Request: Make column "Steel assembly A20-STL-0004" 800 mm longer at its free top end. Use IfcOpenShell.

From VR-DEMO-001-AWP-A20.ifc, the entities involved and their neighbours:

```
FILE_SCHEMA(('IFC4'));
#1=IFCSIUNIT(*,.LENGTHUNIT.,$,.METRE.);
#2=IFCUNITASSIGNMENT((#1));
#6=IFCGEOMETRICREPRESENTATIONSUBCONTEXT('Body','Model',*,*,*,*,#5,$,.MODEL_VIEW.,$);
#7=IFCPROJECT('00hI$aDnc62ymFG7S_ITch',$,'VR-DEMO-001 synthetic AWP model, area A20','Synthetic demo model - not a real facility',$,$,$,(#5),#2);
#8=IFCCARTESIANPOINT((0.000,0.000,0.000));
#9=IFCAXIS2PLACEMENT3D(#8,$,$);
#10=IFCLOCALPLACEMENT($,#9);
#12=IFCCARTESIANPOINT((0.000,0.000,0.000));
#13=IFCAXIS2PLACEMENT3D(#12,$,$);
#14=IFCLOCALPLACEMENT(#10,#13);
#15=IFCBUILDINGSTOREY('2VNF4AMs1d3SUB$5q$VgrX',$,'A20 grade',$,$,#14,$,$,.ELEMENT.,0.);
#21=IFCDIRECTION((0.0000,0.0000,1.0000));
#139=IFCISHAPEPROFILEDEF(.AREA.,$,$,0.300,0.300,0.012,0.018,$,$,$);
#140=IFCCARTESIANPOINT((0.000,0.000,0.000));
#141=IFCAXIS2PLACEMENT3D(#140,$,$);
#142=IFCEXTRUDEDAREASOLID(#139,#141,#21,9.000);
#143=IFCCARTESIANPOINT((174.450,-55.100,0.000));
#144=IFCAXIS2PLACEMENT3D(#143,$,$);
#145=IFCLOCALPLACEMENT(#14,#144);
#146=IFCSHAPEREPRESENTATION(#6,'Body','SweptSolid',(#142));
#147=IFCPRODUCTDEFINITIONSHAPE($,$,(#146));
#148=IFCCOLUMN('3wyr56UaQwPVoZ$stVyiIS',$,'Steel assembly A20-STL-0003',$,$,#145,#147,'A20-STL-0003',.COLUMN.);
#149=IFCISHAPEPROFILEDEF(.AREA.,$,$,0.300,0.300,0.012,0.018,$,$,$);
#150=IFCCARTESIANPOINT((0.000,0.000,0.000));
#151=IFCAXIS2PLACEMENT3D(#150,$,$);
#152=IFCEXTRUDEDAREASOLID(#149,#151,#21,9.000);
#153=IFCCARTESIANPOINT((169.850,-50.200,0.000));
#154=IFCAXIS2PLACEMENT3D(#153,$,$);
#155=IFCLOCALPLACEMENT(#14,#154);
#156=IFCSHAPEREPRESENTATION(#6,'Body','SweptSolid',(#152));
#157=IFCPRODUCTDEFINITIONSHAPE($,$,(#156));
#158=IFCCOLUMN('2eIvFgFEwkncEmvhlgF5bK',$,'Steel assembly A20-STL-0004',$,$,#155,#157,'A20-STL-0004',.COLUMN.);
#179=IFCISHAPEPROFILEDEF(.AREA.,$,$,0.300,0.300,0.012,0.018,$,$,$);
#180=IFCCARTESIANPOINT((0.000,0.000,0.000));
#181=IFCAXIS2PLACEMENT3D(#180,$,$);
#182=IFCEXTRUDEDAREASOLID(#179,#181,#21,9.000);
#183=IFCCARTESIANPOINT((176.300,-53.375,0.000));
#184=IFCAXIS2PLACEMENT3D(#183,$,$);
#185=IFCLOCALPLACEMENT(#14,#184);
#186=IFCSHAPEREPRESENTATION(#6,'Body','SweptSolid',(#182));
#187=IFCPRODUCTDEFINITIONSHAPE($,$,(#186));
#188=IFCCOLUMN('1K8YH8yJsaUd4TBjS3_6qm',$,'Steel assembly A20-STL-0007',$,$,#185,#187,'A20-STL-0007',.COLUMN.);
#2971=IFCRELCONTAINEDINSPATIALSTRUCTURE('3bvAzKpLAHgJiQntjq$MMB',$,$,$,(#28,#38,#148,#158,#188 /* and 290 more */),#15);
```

```python
import ifcopenshell
import ifcopenshell.util.representation

model = ifcopenshell.open("VR-DEMO-001-AWP-A20.ifc")

member = model.by_guid("2eIvFgFEwkncEmvhlgF5bK")
change = 0.8

# The extrusion runs towards the end named, so only its depth changes.
body = ifcopenshell.util.representation.get_representation(member, "Model", "Body")
solid = body.Items[0]
old_length = solid.Depth
solid.Depth += change

print(f"length {old_length:g} -> {solid.Depth:g}")

model.write("VR-DEMO-001-AWP-A20-out.ifc")
```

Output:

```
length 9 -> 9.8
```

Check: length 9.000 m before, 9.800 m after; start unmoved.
